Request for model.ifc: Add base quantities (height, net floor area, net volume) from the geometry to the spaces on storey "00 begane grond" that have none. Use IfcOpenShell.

First a look at what the model holds.

```python
import ifcopenshell
import ifcopenshell.util.element
import ifcopenshell.util.unit

model = ifcopenshell.open("model.ifc")
print(model.schema)
for unit_type in ("LENGTHUNIT", "AREAUNIT", "VOLUMEUNIT"):
    print(unit_type, ifcopenshell.util.unit.calculate_unit_scale(model, unit_type))
storey = next(s for s in model.by_type("IfcBuildingStorey") if s.Name == "00 begane grond")
spaces = [e for e in ifcopenshell.util.element.get_decomposition(storey) if e.is_a("IfcSpace")]
for e in sorted(spaces, key=lambda e: e.id()):
    print(e.id(), e.is_a(), e.Name, list(ifcopenshell.util.element.get_psets(e, qtos_only=True)), sep=" | ")
```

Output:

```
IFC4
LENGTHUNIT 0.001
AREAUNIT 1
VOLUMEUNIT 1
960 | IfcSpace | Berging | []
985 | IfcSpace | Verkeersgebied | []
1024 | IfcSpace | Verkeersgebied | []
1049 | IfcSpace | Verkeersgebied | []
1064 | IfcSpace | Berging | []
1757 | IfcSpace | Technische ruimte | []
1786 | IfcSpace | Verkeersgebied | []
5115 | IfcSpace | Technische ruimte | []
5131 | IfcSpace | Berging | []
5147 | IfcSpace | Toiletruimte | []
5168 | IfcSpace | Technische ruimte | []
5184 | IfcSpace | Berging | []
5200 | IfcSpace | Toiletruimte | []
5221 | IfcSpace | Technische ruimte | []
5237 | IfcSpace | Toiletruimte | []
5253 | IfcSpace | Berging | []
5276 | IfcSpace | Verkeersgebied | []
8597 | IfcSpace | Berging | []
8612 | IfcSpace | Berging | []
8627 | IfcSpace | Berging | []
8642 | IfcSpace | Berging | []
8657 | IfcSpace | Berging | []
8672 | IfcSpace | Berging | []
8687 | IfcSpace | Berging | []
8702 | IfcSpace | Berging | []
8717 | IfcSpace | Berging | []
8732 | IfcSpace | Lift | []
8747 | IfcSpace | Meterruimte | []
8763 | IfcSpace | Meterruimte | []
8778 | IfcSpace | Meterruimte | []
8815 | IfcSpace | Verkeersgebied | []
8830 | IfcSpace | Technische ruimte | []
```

```python
import ifcopenshell
import ifcopenshell.api.pset
import ifcopenshell.geom
import ifcopenshell.util.element
import ifcopenshell.util.shape
import ifcopenshell.util.unit

model = ifcopenshell.open("model.ifc")
unit_scale = ifcopenshell.util.unit.calculate_unit_scale(model)
area_scale = ifcopenshell.util.unit.calculate_unit_scale(model, "AREAUNIT")
volume_scale = ifcopenshell.util.unit.calculate_unit_scale(model, "VOLUMEUNIT")
settings = ifcopenshell.geom.settings()

storey = next(s for s in model.by_type("IfcBuildingStorey") if s.Name == "00 begane grond")
spaces = [e for e in ifcopenshell.util.element.get_decomposition(storey) if e.is_a("IfcSpace")]

for e in sorted(spaces, key=lambda e: e.id()):
    if ifcopenshell.util.element.get_psets(e, qtos_only=True, should_inherit=False):
        continue
    # Geometry comes back in metres, in the element's own axes.
    shape = ifcopenshell.geom.create_shape(settings, e)
    values = {
        "Height": ifcopenshell.util.shape.get_z(shape.geometry) / unit_scale,
        "NetFloorArea": ifcopenshell.util.shape.get_footprint_area(shape.geometry) / area_scale,
        "NetVolume": ifcopenshell.util.shape.get_volume(shape.geometry) / volume_scale,
    }
    qto = ifcopenshell.api.pset.add_qto(model, product=e, name="Qto_SpaceBaseQuantities")
    ifcopenshell.api.pset.edit_qto(model, qto=qto, properties=values)
    print(e.id(), {k: round(v, 3) for k, v in values.items()})

model.write("model_v2.ifc")
```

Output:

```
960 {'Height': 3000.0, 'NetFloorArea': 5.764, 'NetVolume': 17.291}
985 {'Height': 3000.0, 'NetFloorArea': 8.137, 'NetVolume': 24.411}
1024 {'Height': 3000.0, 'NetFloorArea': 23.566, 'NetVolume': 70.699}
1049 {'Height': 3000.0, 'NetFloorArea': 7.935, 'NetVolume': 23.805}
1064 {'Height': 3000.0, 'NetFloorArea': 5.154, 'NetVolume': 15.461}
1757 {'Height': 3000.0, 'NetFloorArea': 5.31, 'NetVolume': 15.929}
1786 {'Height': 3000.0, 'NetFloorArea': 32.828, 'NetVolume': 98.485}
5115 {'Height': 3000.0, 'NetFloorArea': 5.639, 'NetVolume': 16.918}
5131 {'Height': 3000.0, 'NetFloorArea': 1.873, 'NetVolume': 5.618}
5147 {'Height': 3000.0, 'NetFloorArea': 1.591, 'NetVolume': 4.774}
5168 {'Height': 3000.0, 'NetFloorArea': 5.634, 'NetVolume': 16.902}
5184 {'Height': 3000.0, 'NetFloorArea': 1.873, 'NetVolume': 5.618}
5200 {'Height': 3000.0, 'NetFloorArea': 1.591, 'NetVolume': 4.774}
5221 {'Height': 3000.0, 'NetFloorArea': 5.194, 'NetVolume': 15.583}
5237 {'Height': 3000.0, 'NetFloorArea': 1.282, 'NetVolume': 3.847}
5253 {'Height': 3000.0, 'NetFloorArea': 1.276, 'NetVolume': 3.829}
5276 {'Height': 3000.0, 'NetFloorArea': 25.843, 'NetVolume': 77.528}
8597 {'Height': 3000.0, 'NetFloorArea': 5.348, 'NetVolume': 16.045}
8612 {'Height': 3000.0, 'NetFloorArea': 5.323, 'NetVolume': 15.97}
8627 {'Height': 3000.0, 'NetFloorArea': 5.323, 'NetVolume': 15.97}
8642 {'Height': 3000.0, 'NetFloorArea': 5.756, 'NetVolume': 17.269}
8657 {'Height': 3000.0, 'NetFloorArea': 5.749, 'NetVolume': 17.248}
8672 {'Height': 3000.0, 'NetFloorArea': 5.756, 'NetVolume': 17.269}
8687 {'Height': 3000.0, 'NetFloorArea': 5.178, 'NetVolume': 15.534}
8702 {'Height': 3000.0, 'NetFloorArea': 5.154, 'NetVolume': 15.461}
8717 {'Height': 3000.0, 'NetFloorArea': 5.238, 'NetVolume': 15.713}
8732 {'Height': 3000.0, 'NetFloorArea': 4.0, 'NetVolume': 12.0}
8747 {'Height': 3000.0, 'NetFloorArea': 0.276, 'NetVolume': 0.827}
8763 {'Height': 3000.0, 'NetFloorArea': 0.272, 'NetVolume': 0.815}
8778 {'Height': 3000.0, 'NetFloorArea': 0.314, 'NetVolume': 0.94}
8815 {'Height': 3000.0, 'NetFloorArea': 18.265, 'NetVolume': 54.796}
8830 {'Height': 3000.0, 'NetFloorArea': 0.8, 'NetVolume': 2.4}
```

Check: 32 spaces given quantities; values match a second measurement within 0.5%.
